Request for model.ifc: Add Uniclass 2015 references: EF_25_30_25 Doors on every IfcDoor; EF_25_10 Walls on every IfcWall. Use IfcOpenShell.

First a look at what the model holds.

```python
import ifcopenshell

model = ifcopenshell.open("model.ifc")
print(model.schema)
print("classifications:", [c.Name for c in model.by_type("IfcClassification")])
for ifc_class in ("IfcDoor", "IfcRoof", "IfcStair", "IfcWall", "IfcWindow"):
    print(ifc_class, len(model.by_type(ifc_class)))
```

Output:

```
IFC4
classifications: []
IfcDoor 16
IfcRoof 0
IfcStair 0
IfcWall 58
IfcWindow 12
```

```python
import ifcopenshell
import ifcopenshell.api.classification

model = ifcopenshell.open("model.ifc")

system = ifcopenshell.api.classification.add_classification(model, classification="Uniclass 2015")

codes = {
    "IfcDoor": ("EF_25_30_25", "Doors"),
    "IfcWall": ("EF_25_10", "Walls"),
}
for ifc_class, (code, name) in codes.items():
    products = model.by_type(ifc_class)
    ifcopenshell.api.classification.add_reference(
        model, products=products, classification=system, identification=code, name=name
    )
    print(code, len(products))

model.write("model_rev.ifc")
```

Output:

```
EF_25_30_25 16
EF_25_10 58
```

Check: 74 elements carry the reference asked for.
